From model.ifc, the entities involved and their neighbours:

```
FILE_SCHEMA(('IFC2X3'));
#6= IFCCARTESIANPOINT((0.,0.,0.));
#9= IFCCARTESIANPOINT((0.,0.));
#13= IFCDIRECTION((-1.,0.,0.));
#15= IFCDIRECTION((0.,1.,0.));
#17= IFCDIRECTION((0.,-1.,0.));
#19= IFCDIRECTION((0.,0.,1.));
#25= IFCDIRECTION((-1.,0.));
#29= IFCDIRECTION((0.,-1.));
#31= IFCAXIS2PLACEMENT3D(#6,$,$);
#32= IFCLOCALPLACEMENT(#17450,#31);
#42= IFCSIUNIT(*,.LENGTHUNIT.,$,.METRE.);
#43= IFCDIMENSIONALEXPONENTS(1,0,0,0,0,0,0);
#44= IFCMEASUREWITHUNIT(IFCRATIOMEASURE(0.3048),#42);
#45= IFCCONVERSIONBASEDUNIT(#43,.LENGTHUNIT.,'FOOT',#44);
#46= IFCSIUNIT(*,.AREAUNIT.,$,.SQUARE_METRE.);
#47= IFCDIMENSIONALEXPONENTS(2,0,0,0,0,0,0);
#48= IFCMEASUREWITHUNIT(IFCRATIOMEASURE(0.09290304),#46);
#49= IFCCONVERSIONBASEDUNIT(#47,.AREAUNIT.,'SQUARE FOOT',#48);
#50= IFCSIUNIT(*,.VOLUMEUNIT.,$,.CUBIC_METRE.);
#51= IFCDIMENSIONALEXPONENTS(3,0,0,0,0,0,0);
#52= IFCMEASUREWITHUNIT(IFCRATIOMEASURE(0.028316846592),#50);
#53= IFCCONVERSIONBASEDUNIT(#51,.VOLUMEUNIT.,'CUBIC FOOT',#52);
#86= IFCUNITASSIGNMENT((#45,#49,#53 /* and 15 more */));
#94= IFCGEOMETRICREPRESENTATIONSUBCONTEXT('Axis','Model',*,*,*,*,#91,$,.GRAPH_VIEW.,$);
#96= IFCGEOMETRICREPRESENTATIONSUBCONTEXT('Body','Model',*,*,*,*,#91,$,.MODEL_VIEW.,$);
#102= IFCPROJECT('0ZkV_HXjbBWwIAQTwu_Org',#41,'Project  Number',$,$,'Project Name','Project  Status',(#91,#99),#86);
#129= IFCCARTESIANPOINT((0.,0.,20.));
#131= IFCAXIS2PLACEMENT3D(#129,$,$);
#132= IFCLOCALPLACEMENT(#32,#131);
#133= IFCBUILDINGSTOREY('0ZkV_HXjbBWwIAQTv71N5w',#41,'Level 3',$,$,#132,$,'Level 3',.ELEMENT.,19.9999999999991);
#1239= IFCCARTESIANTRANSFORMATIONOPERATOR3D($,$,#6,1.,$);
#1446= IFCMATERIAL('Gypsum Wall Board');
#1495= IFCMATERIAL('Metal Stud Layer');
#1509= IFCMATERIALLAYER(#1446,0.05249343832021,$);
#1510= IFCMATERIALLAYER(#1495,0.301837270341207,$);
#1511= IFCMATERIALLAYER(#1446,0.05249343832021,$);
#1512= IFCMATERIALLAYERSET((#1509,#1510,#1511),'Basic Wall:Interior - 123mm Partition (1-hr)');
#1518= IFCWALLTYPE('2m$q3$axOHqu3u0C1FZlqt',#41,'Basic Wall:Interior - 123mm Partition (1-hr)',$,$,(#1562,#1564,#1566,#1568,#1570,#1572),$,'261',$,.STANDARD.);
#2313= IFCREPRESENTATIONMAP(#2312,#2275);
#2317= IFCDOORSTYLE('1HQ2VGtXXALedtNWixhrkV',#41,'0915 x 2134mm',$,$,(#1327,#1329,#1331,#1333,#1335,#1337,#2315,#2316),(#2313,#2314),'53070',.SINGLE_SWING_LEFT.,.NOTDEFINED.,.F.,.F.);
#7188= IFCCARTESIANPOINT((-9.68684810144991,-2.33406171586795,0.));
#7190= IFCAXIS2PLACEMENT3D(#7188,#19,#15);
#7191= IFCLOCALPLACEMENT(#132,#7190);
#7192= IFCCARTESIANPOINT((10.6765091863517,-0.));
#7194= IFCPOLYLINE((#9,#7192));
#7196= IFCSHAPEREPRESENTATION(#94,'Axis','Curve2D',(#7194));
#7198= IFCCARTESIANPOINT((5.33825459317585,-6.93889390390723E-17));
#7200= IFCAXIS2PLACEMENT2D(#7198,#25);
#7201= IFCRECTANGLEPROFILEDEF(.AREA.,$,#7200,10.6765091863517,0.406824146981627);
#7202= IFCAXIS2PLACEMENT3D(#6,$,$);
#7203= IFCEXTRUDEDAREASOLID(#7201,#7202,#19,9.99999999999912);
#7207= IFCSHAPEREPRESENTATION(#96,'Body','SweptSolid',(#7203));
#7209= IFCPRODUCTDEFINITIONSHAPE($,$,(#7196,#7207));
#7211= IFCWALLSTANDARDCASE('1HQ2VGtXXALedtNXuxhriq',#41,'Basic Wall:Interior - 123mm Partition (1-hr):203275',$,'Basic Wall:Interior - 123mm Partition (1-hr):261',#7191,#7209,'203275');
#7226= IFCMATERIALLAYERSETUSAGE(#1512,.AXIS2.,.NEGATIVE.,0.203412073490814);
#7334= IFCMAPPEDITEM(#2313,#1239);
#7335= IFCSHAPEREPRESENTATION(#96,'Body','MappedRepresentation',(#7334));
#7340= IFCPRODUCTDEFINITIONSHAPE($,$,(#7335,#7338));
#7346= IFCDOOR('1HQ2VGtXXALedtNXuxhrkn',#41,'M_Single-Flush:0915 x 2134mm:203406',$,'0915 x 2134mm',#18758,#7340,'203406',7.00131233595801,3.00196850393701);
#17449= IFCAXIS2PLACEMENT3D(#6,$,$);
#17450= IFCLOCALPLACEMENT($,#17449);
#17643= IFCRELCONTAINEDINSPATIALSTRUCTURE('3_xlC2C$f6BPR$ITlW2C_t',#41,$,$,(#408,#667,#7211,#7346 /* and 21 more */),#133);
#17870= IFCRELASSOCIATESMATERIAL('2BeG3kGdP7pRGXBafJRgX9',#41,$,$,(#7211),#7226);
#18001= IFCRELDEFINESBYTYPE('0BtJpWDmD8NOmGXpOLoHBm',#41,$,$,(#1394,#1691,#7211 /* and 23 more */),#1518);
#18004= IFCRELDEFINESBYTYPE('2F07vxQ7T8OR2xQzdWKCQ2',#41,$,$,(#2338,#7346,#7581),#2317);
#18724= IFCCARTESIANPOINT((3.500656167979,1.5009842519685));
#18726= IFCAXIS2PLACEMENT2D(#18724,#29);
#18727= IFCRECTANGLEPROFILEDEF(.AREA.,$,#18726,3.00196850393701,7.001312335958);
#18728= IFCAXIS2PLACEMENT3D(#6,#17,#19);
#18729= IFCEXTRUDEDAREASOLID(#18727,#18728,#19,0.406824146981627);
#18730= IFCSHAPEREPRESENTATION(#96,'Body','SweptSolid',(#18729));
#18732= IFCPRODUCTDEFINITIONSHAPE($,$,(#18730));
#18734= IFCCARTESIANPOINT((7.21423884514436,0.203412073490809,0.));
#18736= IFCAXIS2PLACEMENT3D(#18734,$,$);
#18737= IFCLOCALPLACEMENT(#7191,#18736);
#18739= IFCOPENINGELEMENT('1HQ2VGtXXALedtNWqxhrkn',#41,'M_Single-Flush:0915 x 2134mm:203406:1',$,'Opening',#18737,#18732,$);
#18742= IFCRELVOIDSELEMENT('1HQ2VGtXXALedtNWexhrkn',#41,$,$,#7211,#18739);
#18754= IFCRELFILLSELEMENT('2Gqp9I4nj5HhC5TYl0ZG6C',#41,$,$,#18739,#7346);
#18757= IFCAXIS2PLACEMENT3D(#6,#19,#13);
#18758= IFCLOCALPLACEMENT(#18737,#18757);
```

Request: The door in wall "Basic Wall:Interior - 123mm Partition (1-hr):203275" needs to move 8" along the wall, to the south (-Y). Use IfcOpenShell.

```python
import ifcopenshell
import ifcopenshell.api.geometry
import ifcopenshell.util.placement
import ifcopenshell.util.unit

model = ifcopenshell.open("model.ifc")
unit_scale = ifcopenshell.util.unit.calculate_unit_scale(model)

door = model.by_guid("1HQ2VGtXXALedtNXuxhrkn")
opening = door.FillsVoids[0].RelatingOpeningElement
wall = opening.VoidsElements[0].RelatingBuildingElement

wall_matrix = ifcopenshell.util.placement.get_local_placement(wall.ObjectPlacement)
shift = wall_matrix[:3, 0] * -8 * 0.0254 / unit_scale
before = ifcopenshell.util.placement.get_local_placement(door.ObjectPlacement)[:3, 3].copy()

# The door is placed relative to its opening, so it follows when the opening moves.
matrix = ifcopenshell.util.placement.get_local_placement(opening.ObjectPlacement)
matrix[:3, 3] += shift
ifcopenshell.api.geometry.edit_object_placement(
    model, product=opening, matrix=matrix, is_si=False, should_transform_children=True
)

after = ifcopenshell.util.placement.get_local_placement(door.ObjectPlacement)[:3, 3]
print("door moved by", (after - before).round(3) + 0.0)

model.write("model_updated.ifc")
```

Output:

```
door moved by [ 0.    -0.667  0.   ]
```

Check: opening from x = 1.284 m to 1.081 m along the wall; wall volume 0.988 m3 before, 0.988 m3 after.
